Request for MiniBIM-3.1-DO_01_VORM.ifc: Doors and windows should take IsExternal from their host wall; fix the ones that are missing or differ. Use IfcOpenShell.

First a look at what the model holds.

```python
import ifcopenshell
import ifcopenshell.util.element

model = ifcopenshell.open("MiniBIM-3.1-DO_01_VORM.ifc")
print(model.schema)
seen = {}
for e in model.by_type("IfcDoor") + model.by_type("IfcWindow"):
    if not e.FillsVoids:
        continue
    host = e.FillsVoids[0].RelatingOpeningElement.VoidsElements[0].RelatingBuildingElement
    own = ifcopenshell.util.element.get_pset(e, f"Pset_{e.is_a()[3:].removesuffix('StandardCase')}Common", "IsExternal")
    wall = ifcopenshell.util.element.get_pset(host, "Pset_WallCommon", "IsExternal")
    seen[e.is_a(), own, wall] = seen.get((e.is_a(), own, wall), 0) + 1
for (cls, own, wall), count in sorted(seen.items(), key=str):
    print(count, cls, "IsExternal:", own, "| host wall:", wall)
```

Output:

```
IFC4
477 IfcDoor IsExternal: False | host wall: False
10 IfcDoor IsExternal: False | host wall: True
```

```python
import ifcopenshell
import ifcopenshell.api.pset
import ifcopenshell.util.element

model = ifcopenshell.open("MiniBIM-3.1-DO_01_VORM.ifc")

count = 0
for ifc_class, pset_name in (("IfcDoor", "Pset_DoorCommon"), ("IfcWindow", "Pset_WindowCommon")):
    for e in model.by_type(ifc_class):
        if not e.FillsVoids:
            continue
        host = e.FillsVoids[0].RelatingOpeningElement.VoidsElements[0].RelatingBuildingElement
        external = ifcopenshell.util.element.get_pset(host, "Pset_WallCommon", "IsExternal")
        if external is None or ifcopenshell.util.element.get_pset(e, pset_name, "IsExternal") == external:
            continue
        pset = ifcopenshell.api.pset.add_pset(model, product=e, name=pset_name)
        ifcopenshell.api.pset.edit_pset(model, pset=pset, properties={"IsExternal": external})
        count += 1

print(count, "updated")

model.write("MiniBIM-3.1-DO_01_VORM_rev.ifc")
```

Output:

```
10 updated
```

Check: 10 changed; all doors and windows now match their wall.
